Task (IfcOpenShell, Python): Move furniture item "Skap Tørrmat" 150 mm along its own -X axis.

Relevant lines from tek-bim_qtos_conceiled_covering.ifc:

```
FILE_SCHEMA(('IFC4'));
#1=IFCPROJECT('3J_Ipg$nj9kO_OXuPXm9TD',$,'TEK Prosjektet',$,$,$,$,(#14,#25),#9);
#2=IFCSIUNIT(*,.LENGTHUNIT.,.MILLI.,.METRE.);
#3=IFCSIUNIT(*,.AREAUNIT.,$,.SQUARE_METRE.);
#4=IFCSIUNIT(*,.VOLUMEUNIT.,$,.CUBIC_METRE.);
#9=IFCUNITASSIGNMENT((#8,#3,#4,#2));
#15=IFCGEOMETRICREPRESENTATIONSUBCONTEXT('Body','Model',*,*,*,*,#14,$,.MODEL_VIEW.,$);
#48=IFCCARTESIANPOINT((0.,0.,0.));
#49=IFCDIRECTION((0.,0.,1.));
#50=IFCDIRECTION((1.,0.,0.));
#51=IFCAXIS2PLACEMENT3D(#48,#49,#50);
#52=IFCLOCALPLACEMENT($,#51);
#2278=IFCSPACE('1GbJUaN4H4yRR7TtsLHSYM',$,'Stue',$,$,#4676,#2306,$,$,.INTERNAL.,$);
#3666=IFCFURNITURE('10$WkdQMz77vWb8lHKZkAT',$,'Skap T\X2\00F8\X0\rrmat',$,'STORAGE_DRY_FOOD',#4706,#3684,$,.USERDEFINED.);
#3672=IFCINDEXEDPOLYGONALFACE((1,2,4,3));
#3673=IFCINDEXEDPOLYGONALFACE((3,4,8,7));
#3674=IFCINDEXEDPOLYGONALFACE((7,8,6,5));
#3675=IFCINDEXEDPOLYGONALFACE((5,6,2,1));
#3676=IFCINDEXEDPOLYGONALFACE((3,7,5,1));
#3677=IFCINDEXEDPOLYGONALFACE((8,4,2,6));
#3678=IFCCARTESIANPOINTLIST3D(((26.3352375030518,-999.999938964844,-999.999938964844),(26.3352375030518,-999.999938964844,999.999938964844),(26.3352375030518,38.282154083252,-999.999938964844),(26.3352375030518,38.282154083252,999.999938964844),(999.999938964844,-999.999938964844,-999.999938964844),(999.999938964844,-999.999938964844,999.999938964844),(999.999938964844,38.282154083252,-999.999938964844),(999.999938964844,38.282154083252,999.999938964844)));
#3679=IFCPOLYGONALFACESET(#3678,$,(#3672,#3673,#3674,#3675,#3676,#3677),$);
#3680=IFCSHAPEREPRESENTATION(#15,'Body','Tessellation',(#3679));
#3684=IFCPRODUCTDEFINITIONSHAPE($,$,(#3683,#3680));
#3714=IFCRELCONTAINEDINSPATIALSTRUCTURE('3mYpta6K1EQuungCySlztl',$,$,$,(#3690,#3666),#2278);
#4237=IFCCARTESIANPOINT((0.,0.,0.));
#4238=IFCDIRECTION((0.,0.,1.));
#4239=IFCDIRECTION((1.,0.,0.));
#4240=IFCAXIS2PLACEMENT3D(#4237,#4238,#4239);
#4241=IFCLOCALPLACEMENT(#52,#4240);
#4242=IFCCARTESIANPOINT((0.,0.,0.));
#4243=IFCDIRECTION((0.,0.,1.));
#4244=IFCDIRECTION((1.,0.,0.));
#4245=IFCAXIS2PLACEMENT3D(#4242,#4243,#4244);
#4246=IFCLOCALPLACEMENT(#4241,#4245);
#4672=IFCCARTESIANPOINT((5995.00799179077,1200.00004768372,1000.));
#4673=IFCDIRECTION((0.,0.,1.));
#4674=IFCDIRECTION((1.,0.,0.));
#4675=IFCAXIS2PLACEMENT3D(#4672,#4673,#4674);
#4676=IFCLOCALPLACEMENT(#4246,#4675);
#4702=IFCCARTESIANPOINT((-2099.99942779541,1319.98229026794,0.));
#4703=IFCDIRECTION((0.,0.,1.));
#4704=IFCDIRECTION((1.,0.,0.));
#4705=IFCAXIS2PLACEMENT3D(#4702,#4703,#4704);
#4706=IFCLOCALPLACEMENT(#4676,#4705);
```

```python
import ifcopenshell
import ifcopenshell.api.geometry
import ifcopenshell.util.placement

model = ifcopenshell.open("tek-bim_qtos_conceiled_covering.ifc")

item = model.by_id(3666)
matrix = ifcopenshell.util.placement.get_local_placement(item.ObjectPlacement)
matrix[:3, 3] -= matrix[:3, 0] * 150.0
ifcopenshell.api.geometry.edit_object_placement(model, product=item, matrix=matrix, is_si=False)

print(ifcopenshell.util.placement.get_local_placement(item.ObjectPlacement).round(3) + 0.0)

model.write("tek-bim_qtos_conceiled_covering_edited.ifc")
```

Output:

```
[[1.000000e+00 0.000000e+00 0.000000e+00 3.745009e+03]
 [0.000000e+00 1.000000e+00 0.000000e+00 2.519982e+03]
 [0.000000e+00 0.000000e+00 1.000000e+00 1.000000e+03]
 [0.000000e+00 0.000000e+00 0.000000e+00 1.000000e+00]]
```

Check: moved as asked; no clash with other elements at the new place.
